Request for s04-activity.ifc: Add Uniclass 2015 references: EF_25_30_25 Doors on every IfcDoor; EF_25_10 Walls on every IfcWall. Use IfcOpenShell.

First a look at what the model holds.

```python
import ifcopenshell

model = ifcopenshell.open("s04-activity.ifc")
print(model.schema)
print("classifications:", [c.Name for c in model.by_type("IfcClassification")])
for ifc_class in ("IfcDoor", "IfcRoof", "IfcStair", "IfcWall", "IfcWindow"):
    print(ifc_class, len(model.by_type(ifc_class)))
```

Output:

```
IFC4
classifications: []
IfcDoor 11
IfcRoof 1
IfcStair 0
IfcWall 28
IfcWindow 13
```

```python
import ifcopenshell
import ifcopenshell.api.classification

model = ifcopenshell.open("s04-activity.ifc")

system = ifcopenshell.api.classification.add_classification(model, classification="Uniclass 2015")

codes = {
    "IfcDoor": ("EF_25_30_25", "Doors"),
    "IfcWall": ("EF_25_10", "Walls"),
}
for ifc_class, (code, name) in codes.items():
    products = model.by_type(ifc_class)
    ifcopenshell.api.classification.add_reference(
        model, products=products, classification=system, identification=code, name=name
    )
    print(code, len(products))

model.write("s04-activity_edited.ifc")
```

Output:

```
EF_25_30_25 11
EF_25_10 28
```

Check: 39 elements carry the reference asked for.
